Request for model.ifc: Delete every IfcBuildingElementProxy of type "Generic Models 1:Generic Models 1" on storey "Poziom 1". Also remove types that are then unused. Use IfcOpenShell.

First a look at what the model holds.

```python
import ifcopenshell
import ifcopenshell.util.element

model = ifcopenshell.open("model.ifc")
print(model.schema)
storey = next(s for s in model.by_type("IfcBuildingStorey") if s.Name == "Poziom 1")
proxies = [e for e in ifcopenshell.util.element.get_decomposition(storey) if e.is_a("IfcBuildingElementProxy")]
seen = {}
for e in proxies:
    element_type = ifcopenshell.util.element.get_type(e)
    name = element_type.Name if element_type not in (None, e) else None
    seen[name] = seen.get(name, 0) + 1
for name, count in sorted(seen.items(), key=str):
    print(count, "x", name)
```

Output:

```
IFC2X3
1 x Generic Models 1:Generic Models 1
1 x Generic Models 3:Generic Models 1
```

```python
import ifcopenshell
import ifcopenshell.api.root
import ifcopenshell.util.element

model = ifcopenshell.open("model.ifc")

storey = next(s for s in model.by_type("IfcBuildingStorey") if s.Name == "Poziom 1")
proxies = [e for e in ifcopenshell.util.element.get_decomposition(storey) if e.is_a("IfcBuildingElementProxy")]
targets = [e for e in proxies if (t := ifcopenshell.util.element.get_type(e)) not in (None, e) and t.Name == "Generic Models 1:Generic Models 1"]
types = {ifcopenshell.util.element.get_type(e) for e in targets} - {None, *targets}

for e in targets:
    ifcopenshell.api.root.remove_product(model, product=e)
print(len(targets), "removed")

unused = [t for t in types if not ifcopenshell.util.element.get_types(t)]
for t in unused:
    ifcopenshell.api.root.remove_product(model, product=t)
print(len(unused), "unused types removed")

model.write("model_v2.ifc")
```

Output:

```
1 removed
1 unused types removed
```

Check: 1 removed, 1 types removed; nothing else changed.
